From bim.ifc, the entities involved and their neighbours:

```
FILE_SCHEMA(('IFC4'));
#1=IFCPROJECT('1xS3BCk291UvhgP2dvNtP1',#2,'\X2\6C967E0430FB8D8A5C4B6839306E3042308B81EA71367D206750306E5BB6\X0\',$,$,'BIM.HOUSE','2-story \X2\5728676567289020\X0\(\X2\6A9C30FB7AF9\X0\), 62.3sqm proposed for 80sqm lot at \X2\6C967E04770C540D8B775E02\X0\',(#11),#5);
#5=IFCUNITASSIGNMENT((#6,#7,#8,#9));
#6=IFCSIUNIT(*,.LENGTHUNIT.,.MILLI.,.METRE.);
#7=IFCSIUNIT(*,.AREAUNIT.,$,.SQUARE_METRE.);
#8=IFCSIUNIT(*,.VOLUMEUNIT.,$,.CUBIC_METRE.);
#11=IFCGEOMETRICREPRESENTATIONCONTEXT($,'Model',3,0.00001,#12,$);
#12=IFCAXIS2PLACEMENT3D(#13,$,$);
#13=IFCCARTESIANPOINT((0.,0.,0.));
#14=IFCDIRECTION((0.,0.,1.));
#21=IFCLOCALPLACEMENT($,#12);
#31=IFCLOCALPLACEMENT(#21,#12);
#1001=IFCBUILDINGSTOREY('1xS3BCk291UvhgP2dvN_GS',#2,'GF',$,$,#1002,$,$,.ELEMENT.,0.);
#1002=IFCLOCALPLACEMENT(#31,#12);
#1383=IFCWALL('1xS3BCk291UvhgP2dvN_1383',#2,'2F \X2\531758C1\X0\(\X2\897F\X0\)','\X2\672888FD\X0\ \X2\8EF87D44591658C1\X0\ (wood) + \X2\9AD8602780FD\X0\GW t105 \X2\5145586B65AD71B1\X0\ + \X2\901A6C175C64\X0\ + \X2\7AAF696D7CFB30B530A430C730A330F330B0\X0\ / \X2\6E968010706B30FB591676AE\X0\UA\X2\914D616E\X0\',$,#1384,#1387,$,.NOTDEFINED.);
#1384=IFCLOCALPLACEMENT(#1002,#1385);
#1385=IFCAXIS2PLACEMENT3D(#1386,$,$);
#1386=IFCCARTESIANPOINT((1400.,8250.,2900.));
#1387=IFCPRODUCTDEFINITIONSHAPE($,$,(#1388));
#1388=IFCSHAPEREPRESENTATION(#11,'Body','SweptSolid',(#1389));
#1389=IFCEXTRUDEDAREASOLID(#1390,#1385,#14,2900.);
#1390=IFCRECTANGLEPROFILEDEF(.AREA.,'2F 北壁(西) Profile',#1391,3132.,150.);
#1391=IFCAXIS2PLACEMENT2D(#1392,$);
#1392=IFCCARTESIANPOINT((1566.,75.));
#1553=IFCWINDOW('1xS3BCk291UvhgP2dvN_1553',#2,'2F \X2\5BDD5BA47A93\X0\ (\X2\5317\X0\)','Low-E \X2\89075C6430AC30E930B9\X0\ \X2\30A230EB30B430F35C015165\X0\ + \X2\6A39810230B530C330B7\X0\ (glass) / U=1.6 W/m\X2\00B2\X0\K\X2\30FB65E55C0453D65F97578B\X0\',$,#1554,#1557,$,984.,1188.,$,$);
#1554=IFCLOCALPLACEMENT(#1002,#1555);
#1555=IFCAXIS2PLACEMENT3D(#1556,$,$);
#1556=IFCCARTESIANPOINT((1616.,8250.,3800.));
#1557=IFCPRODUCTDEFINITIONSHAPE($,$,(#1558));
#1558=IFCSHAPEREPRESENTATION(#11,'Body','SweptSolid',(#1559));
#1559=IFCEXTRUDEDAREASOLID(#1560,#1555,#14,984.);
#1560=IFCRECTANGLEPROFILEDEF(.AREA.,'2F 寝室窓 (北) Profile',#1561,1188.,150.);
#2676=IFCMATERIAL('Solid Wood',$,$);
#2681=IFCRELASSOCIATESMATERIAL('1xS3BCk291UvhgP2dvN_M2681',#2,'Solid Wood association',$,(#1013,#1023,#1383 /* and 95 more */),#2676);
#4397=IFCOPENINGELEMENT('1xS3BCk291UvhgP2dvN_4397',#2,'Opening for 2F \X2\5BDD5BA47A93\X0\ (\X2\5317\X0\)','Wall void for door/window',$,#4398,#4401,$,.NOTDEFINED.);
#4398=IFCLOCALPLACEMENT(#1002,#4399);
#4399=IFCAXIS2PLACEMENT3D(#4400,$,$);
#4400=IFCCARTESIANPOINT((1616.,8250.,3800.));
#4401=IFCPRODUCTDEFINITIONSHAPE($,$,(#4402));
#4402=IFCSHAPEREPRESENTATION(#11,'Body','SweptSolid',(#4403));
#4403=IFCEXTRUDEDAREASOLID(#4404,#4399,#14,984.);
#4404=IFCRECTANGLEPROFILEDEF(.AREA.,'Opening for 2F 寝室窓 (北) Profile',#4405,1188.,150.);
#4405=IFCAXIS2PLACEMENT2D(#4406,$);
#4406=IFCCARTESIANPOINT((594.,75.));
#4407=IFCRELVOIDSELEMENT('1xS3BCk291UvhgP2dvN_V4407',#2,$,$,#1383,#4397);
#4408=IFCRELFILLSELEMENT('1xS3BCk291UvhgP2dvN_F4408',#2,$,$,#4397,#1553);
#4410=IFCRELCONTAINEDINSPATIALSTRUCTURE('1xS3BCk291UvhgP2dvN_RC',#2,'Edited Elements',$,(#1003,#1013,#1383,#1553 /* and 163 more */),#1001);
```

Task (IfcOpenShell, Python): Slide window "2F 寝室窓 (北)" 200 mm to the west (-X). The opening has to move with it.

```python
import ifcopenshell
import ifcopenshell.api.geometry
import ifcopenshell.util.placement

model = ifcopenshell.open("bim.ifc")

window = model.by_guid("1xS3BCk291UvhgP2dvN_1553")
opening = window.FillsVoids[0].RelatingOpeningElement
wall = opening.VoidsElements[0].RelatingBuildingElement

wall_matrix = ifcopenshell.util.placement.get_local_placement(wall.ObjectPlacement)
shift = wall_matrix[:3, 0] * -200.0
before = ifcopenshell.util.placement.get_local_placement(window.ObjectPlacement)[:3, 3].copy()

# The window is not placed relative to its opening, so move both.
for product in (opening, window):
    matrix = ifcopenshell.util.placement.get_local_placement(product.ObjectPlacement)
    matrix[:3, 3] += shift
    ifcopenshell.api.geometry.edit_object_placement(model, product=product, matrix=matrix, is_si=False)

after = ifcopenshell.util.placement.get_local_placement(window.ObjectPlacement)[:3, 3]
print("window moved by", (after - before).round(3) + 0.0)

model.write("bim_rev.ifc")
```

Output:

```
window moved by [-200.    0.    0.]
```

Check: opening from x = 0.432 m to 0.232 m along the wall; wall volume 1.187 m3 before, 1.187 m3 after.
